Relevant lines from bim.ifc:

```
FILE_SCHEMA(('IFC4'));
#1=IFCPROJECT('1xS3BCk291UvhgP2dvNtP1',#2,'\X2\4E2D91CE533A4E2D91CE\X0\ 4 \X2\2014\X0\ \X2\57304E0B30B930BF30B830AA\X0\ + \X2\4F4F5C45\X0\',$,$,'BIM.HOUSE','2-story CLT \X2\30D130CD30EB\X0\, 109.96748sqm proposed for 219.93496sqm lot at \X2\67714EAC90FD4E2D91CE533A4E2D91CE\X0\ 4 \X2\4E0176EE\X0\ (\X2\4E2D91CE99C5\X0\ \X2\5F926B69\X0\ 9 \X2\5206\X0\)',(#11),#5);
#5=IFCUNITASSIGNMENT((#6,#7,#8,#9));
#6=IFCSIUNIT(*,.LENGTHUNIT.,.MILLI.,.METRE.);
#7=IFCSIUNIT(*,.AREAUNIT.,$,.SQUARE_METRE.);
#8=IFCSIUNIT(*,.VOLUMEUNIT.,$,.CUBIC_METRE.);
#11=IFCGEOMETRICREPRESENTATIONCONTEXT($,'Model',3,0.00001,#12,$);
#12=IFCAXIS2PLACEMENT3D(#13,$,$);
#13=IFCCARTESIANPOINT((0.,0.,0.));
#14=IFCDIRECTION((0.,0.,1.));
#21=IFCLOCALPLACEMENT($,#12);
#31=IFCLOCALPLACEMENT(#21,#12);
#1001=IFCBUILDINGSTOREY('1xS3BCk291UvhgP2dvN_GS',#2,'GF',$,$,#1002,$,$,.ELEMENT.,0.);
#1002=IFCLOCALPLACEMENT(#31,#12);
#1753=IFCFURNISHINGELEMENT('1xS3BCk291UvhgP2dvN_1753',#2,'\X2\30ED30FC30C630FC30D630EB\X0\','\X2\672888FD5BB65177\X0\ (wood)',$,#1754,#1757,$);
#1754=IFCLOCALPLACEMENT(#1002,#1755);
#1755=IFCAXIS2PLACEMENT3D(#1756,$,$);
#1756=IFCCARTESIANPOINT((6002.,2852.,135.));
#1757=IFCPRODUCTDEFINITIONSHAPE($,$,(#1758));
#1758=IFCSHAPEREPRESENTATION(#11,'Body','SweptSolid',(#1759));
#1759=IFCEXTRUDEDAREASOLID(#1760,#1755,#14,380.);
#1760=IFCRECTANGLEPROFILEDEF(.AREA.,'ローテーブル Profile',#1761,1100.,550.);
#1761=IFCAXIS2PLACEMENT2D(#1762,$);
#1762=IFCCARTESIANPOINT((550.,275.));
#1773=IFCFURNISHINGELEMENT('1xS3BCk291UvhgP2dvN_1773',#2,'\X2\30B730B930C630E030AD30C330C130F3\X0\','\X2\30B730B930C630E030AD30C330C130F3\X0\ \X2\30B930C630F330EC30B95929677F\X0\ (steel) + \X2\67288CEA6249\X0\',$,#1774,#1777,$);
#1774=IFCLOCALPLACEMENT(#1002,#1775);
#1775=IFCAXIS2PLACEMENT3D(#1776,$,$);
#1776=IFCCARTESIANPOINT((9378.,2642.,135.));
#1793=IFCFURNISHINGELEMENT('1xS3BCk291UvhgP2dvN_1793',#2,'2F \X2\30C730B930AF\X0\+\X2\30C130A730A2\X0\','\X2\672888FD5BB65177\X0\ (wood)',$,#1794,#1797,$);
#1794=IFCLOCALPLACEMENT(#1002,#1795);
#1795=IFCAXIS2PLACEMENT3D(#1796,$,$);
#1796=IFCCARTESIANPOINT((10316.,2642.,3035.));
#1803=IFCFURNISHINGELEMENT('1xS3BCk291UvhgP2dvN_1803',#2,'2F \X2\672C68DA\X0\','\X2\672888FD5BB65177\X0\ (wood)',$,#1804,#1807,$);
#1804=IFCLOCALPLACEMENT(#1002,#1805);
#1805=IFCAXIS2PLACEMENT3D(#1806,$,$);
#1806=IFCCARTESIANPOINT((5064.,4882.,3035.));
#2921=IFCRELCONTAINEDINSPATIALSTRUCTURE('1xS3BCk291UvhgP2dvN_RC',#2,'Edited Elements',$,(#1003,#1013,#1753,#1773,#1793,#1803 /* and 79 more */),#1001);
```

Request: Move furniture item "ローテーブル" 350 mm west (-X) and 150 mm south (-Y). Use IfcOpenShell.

```python
import ifcopenshell
import ifcopenshell.api.geometry
import ifcopenshell.util.placement
import ifcopenshell.util.unit

model = ifcopenshell.open("bim.ifc")
unit_scale = ifcopenshell.util.unit.calculate_unit_scale(model)

item = model.by_id(1753)
matrix = ifcopenshell.util.placement.get_local_placement(item.ObjectPlacement)
matrix[0, 3] -= 0.35 / unit_scale
matrix[1, 3] -= 0.15 / unit_scale
ifcopenshell.api.geometry.edit_object_placement(model, product=item, matrix=matrix, is_si=False)

print(ifcopenshell.util.placement.get_local_placement(item.ObjectPlacement).round(3) + 0.0)

model.write("bim_rev.ifc")
```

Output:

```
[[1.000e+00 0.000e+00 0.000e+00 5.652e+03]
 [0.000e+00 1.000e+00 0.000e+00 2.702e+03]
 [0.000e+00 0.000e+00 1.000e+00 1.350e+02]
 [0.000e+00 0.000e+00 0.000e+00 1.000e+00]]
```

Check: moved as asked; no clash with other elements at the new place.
